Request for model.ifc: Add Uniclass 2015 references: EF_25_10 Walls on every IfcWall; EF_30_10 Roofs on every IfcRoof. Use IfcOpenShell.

First a look at what the model holds.

```python
import ifcopenshell

model = ifcopenshell.open("model.ifc")
print(model.schema)
print("classifications:", [c.Name for c in model.by_type("IfcClassification")])
for ifc_class in ("IfcDoor", "IfcRoof", "IfcStair", "IfcWall", "IfcWindow"):
    print(ifc_class, len(model.by_type(ifc_class)))
```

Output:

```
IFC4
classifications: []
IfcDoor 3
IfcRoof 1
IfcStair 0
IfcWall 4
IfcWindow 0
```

```python
import ifcopenshell
import ifcopenshell.api.classification

model = ifcopenshell.open("model.ifc")

system = ifcopenshell.api.classification.add_classification(model, classification="Uniclass 2015")

codes = {
    "IfcWall": ("EF_25_10", "Walls"),
    "IfcRoof": ("EF_30_10", "Roofs"),
}
for ifc_class, (code, name) in codes.items():
    products = model.by_type(ifc_class)
    ifcopenshell.api.classification.add_reference(
        model, products=products, classification=system, identification=code, name=name
    )
    print(code, len(products))

model.write("model_v2.ifc")
```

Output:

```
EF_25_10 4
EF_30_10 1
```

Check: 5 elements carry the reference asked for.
